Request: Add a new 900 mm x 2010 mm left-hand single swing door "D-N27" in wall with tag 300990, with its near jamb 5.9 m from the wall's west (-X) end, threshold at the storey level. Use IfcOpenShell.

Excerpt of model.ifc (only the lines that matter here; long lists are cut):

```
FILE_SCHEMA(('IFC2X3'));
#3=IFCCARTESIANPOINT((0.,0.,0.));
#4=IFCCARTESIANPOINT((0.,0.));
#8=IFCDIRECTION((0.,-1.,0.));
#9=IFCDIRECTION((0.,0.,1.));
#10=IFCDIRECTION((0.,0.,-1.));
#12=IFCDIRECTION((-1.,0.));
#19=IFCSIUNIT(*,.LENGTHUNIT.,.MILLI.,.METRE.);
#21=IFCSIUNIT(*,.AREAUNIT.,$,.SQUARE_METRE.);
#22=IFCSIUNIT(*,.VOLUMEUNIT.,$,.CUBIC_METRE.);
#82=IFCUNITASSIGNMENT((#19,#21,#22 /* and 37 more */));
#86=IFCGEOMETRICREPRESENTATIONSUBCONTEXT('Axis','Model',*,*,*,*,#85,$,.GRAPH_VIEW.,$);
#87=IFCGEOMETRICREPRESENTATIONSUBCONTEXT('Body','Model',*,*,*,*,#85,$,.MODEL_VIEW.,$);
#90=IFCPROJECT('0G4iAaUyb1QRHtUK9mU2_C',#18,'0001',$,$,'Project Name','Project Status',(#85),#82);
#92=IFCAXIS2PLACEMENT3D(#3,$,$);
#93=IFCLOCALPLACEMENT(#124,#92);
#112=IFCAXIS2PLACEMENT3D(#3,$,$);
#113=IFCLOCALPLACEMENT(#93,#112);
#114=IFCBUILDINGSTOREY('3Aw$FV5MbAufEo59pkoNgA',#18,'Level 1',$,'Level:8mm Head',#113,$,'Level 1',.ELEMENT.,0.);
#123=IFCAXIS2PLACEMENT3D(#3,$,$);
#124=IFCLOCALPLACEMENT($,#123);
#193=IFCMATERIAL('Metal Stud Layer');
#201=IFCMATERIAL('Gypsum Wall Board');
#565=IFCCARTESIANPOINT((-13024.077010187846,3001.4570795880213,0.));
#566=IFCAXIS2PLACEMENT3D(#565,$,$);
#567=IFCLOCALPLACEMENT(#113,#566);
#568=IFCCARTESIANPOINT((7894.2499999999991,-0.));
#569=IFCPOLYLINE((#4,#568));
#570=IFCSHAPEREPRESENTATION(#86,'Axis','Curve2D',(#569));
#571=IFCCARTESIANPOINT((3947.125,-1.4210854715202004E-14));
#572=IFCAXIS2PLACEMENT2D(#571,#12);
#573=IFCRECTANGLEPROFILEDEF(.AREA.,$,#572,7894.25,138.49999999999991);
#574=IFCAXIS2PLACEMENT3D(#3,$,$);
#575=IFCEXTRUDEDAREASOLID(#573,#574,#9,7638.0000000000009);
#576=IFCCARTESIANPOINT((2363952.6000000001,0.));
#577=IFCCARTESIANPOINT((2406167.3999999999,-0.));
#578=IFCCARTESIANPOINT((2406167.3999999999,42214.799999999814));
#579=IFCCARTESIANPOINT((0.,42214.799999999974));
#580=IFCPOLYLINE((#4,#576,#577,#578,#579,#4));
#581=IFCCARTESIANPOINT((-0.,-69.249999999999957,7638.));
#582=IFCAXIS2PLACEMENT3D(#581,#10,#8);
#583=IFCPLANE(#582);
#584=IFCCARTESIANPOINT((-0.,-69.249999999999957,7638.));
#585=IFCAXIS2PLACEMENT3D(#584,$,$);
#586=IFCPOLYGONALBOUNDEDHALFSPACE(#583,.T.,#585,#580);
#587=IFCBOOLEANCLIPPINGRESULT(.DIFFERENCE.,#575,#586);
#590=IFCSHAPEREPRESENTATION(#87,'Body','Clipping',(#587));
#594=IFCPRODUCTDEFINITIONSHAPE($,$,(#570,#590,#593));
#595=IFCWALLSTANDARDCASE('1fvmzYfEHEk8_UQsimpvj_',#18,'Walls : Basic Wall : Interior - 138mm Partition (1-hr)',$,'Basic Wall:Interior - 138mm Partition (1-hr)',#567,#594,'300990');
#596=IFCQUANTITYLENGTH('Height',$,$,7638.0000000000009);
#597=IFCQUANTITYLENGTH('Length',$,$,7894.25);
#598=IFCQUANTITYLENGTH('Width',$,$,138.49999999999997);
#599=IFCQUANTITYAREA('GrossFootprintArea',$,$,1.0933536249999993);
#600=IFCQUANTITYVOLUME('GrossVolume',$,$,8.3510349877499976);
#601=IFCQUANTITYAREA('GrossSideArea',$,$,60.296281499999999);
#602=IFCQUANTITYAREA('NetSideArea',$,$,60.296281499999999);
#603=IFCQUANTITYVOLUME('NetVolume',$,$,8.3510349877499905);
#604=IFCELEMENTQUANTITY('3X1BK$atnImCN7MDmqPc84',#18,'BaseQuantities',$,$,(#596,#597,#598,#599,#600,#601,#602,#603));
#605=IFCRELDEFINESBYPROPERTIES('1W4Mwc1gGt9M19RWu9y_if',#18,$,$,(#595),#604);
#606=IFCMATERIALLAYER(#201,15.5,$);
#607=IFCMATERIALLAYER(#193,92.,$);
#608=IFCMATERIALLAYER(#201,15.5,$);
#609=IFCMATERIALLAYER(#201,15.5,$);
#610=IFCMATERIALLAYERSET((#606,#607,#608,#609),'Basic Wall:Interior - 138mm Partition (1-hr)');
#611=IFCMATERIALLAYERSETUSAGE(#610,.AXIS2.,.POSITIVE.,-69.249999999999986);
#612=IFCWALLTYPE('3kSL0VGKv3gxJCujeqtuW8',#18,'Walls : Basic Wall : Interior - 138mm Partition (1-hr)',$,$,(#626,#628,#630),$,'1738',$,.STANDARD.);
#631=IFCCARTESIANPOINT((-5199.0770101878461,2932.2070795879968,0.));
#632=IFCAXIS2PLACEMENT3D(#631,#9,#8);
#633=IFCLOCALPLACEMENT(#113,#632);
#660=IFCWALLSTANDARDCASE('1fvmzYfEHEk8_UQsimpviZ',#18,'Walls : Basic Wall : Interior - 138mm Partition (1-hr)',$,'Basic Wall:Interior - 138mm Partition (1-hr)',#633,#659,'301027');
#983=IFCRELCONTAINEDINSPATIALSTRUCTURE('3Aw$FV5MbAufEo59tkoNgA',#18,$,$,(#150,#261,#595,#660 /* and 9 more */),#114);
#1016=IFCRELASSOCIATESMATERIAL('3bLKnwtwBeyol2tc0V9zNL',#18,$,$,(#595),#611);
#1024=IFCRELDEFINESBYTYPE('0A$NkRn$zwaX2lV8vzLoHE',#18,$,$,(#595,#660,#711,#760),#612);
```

```python
import numpy as np
import ifcopenshell
import ifcopenshell.api.feature
import ifcopenshell.api.geometry
import ifcopenshell.api.pset
import ifcopenshell.api.root
import ifcopenshell.api.spatial
import ifcopenshell.api.type
import ifcopenshell.geom
import ifcopenshell.util.element
import ifcopenshell.util.placement
import ifcopenshell.util.representation
import ifcopenshell.util.shape
import ifcopenshell.util.unit

model = ifcopenshell.open("model.ifc")
unit_scale = ifcopenshell.util.unit.calculate_unit_scale(model)
area_scale = ifcopenshell.util.unit.calculate_unit_scale(model, "AREAUNIT")
volume_scale = ifcopenshell.util.unit.calculate_unit_scale(model, "VOLUMEUNIT")
settings = ifcopenshell.geom.settings()


def volume(element):
    """Net volume in cubic metres, openings subtracted."""
    shape = ifcopenshell.geom.create_shape(settings, element)
    return ifcopenshell.util.shape.get_volume(shape.geometry)


wall = model.by_guid("1fvmzYfEHEk8_UQsimpvj_")
storey = ifcopenshell.util.element.get_container(wall, ifc_class="IfcBuildingStorey")
context = ifcopenshell.util.representation.get_context(model, "Model", "Body", "MODEL_VIEW")
before = volume(wall)

width, height, from_end, sill = 0.9, 2.01, 5.9, 0.0  # metres

# The wall runs along its own X axis, and the end named is its -X end.
wall_shape = ifcopenshell.geom.create_shape(settings, wall)
x, y, z = ifcopenshell.util.shape.get_vertices(wall_shape.geometry).T
start = x.min() + from_end
face, thickness = float(y.min()), float(y.max() - y.min())
wall_matrix = ifcopenshell.util.placement.get_local_placement(wall.ObjectPlacement)
level = ifcopenshell.util.placement.get_local_placement(storey.ObjectPlacement)[2, 3]


def in_wall(x, y):
    """Placement at x, y metres in the wall's axes, at sill height."""
    matrix = wall_matrix.copy()
    matrix[:, 3] = wall_matrix @ np.array([x / unit_scale, y / unit_scale, 0.0, 1.0])
    matrix[2, 3] = level + sill / unit_scale
    return matrix


# Opening: a box that overshoots both wall faces by 50 mm.
opening = ifcopenshell.api.root.create_entity(model, ifc_class="IfcOpeningElement")
box = ifcopenshell.api.geometry.add_wall_representation(
    model, context=context, length=width, height=height, thickness=thickness + 0.1
)
ifcopenshell.api.geometry.assign_representation(model, product=opening, representation=box)
ifcopenshell.api.geometry.edit_object_placement(model, product=opening, matrix=in_wall(start, face - 0.05), is_si=False)
ifcopenshell.api.feature.add_feature(model, feature=opening, element=wall)

door = ifcopenshell.api.root.create_entity(model, ifc_class="IfcDoor", name="D-N27")
door.OverallWidth, door.OverallHeight = width / unit_scale, height / unit_scale
body = ifcopenshell.api.geometry.add_door_representation(
    model,
    context=context,
    overall_width=door.OverallWidth,
    overall_height=door.OverallHeight,
    operation_type="SINGLE_SWING_LEFT",
    lining_properties={"LiningDepth": thickness / unit_scale, "ThresholdDepth": thickness / unit_scale},
)
ifcopenshell.api.geometry.assign_representation(model, product=door, representation=body)
ifcopenshell.api.spatial.assign_container(model, products=[door], relating_structure=storey)
fills = ifcopenshell.api.feature.add_filling(model, opening=opening, element=door)
fills.OwnerHistory = door.OwnerHistory  # required in IFC2X3

# IFC2X3 keeps the operation on the door style.
style = ifcopenshell.api.root.create_entity(model, ifc_class="IfcDoorStyle", name="D-N27")
style.OperationType, style.ConstructionType = "SINGLE_SWING_LEFT", "NOTDEFINED"
style.ParameterTakesPrecedence = style.Sizeable = False
ifcopenshell.api.type.assign_type(model, related_objects=[door], relating_type=style)

# The lining spans the wall, so the door starts at the wall face.
ifcopenshell.api.geometry.edit_object_placement(model, product=door, matrix=in_wall(start, face), is_si=False)

after = volume(wall)

# Update the wall's stored quantities.
qto = model.by_id(ifcopenshell.util.element.get_pset(wall, "BaseQuantities", should_inherit=False)["id"])
ifcopenshell.api.pset.edit_qto(model, qto=qto, properties={
    "NetSideArea": after / thickness / area_scale,
    "NetVolume": after / volume_scale,
})

print(f"wall volume {before:.3f} -> {after:.3f} m3")

model.write("model_v2.ifc")
```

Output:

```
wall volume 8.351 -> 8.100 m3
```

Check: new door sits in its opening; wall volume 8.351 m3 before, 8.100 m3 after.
